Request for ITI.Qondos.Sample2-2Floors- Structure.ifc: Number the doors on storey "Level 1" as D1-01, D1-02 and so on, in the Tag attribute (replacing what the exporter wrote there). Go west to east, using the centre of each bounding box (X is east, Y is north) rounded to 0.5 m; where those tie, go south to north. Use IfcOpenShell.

First a look at what the model holds.

```python
import ifcopenshell
import ifcopenshell.util.element
import ifcopenshell.util.placement

model = ifcopenshell.open("ITI.Qondos.Sample2-2Floors- Structure.ifc")
print(model.schema)
storey = next(s for s in model.by_type("IfcBuildingStorey") if s.Name == "Level 1")
doors = [e for e in ifcopenshell.util.element.get_decomposition(storey) if e.is_a("IfcDoor")]
for e in sorted(doors, key=lambda e: e.id()):
    origin = ifcopenshell.util.placement.get_local_placement(e.ObjectPlacement)[:3, 3]
    print(e.id(), e.Tag, e.Name, origin.round(2) + 0.0, sep=" | ")
```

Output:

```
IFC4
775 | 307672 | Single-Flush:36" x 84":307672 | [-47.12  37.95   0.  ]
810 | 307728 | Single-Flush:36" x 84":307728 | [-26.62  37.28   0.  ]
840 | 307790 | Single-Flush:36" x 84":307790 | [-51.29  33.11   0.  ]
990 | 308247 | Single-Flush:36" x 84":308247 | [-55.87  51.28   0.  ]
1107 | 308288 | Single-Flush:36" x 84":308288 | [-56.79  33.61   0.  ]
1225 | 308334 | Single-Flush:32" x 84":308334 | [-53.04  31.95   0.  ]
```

```python
import ifcopenshell
import ifcopenshell.geom
import ifcopenshell.util.element
import ifcopenshell.util.shape

model = ifcopenshell.open("ITI.Qondos.Sample2-2Floors- Structure.ifc")
settings = ifcopenshell.geom.settings()
settings.set("use-world-coords", True)


def centre(element):
    shape = ifcopenshell.geom.create_shape(settings, element)
    return ifcopenshell.util.shape.get_bbox_centroid(shape.geometry)


storey = next(s for s in model.by_type("IfcBuildingStorey") if s.Name == "Level 1")
doors = [e for e in ifcopenshell.util.element.get_decomposition(storey) if e.is_a("IfcDoor")]

# Insertion points can sit at a corner or the storey origin, so sort by the geometry (in metres).
centres = {e: centre(e) for e in doors}
doors.sort(key=lambda e: (round(centres[e][0] / 0.5), centres[e][1]))

for i, e in enumerate(doors, start=1):
    number = f"D1-{i:02d}"
    e.Tag = number
    print(e.id(), number)

model.write("ITI.Qondos.Sample2-2Floors- Structure-out.ifc")
```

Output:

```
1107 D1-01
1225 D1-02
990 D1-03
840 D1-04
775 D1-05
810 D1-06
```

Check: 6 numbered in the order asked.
